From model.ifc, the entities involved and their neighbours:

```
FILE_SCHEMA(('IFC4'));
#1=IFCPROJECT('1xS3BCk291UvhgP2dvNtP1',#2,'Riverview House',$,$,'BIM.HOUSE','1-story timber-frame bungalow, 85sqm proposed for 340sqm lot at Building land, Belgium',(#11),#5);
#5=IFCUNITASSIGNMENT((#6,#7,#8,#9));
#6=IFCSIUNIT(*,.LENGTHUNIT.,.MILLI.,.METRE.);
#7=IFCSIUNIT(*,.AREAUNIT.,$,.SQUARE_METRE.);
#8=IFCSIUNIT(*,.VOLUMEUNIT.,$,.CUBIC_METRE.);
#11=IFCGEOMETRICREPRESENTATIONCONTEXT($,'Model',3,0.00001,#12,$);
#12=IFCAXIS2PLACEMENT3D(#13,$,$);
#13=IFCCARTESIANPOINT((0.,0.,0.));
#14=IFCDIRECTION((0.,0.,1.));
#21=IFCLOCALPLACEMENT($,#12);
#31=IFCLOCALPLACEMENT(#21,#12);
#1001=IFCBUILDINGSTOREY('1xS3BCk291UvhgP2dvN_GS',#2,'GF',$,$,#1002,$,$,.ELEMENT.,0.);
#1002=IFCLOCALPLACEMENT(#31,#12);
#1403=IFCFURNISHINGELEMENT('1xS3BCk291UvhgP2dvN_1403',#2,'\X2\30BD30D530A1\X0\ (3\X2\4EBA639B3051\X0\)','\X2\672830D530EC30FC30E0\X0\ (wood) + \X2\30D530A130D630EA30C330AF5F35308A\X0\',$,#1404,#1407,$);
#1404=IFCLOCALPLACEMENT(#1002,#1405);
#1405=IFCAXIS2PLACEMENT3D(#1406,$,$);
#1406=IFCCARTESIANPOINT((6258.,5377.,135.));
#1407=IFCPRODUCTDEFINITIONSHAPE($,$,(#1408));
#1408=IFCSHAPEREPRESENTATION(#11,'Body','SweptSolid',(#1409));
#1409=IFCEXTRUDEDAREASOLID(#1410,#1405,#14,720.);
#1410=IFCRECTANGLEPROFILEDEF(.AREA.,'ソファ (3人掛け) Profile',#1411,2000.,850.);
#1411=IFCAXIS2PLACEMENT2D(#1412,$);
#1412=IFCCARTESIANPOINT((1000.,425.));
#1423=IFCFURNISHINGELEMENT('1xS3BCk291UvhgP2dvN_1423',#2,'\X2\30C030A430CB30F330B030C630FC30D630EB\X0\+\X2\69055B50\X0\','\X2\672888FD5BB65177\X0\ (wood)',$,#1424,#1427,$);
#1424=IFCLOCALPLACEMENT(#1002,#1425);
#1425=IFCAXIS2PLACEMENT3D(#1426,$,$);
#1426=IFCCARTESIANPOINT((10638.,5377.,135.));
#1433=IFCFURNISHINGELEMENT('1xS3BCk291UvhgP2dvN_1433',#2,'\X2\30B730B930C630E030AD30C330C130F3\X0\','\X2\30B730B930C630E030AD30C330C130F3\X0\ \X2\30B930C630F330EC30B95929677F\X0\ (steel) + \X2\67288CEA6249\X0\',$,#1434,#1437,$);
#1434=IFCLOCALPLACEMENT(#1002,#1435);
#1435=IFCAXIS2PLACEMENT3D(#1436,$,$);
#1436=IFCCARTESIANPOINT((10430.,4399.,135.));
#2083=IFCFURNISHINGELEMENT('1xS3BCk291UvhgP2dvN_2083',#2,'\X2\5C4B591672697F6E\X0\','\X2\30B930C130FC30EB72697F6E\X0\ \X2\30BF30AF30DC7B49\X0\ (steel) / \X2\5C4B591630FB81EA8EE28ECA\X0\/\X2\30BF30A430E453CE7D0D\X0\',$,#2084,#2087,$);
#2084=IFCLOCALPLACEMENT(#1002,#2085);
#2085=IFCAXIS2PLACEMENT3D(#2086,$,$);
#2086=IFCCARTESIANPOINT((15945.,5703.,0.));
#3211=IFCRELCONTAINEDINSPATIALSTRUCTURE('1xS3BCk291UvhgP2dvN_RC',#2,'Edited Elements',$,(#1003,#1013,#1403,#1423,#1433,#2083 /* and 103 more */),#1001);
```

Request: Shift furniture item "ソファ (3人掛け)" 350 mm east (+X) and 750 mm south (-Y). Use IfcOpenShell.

```python
import ifcopenshell
import ifcopenshell.api.geometry
import ifcopenshell.util.placement

model = ifcopenshell.open("model.ifc")

item = model.by_guid("1xS3BCk291UvhgP2dvN_1403")
matrix = ifcopenshell.util.placement.get_local_placement(item.ObjectPlacement)
matrix[0, 3] += 350.0
matrix[1, 3] -= 750.0
ifcopenshell.api.geometry.edit_object_placement(model, product=item, matrix=matrix, is_si=False)

print(ifcopenshell.util.placement.get_local_placement(item.ObjectPlacement).round(3) + 0.0)

model.write("model_rev.ifc")
```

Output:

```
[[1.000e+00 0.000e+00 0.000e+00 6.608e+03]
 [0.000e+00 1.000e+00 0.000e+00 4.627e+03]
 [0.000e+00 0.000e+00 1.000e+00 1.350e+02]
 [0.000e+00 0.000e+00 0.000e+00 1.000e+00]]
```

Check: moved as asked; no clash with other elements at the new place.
